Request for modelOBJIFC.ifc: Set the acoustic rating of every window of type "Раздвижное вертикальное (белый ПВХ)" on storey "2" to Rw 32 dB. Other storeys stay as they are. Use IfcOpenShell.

First a look at what the model holds.

```python
import ifcopenshell
import ifcopenshell.util.element

model = ifcopenshell.open("modelOBJIFC.ifc")
print(model.schema)
storey = next(s for s in model.by_type("IfcBuildingStorey") if s.Name == "2")
windows = [e for e in ifcopenshell.util.element.get_decomposition(storey) if e.is_a("IfcWindow")]
seen = {}
for e in windows:
    element_type = ifcopenshell.util.element.get_type(e)
    key = (element_type.Name if element_type != e and element_type else None, ifcopenshell.util.element.get_pset(e, "Pset_WindowCommon", "AcousticRating"))
    seen[key] = seen.get(key, 0) + 1
for (name, value), count in sorted(seen.items(), key=str):
    print(count, "x", name, "|", value)
```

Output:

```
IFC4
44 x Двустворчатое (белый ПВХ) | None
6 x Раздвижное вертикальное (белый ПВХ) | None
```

```python
import ifcopenshell
import ifcopenshell.api.pset
import ifcopenshell.util.element

model = ifcopenshell.open("modelOBJIFC.ifc")

storey = next(s for s in model.by_type("IfcBuildingStorey") if s.Name == "2")
windows = [e for e in ifcopenshell.util.element.get_decomposition(storey) if e.is_a("IfcWindow")]

count = 0
for e in windows:
    element_type = ifcopenshell.util.element.get_type(e)
    if element_type in (None, e) or element_type.Name != "Раздвижное вертикальное (белый ПВХ)":
        continue
    # add_pset returns the element's existing set when there is one.
    pset = ifcopenshell.api.pset.add_pset(model, product=e, name="Pset_WindowCommon")
    ifcopenshell.api.pset.edit_pset(model, pset=pset, properties={"AcousticRating": "Rw 32 dB"})
    count += 1

print(count, "windows updated")

model.write("modelOBJIFC_rev.ifc")
```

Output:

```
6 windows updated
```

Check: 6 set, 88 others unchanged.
